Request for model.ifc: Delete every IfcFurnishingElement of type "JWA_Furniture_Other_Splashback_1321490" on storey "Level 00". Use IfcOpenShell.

First a look at what the model holds.

```python
import ifcopenshell
import ifcopenshell.util.element

model = ifcopenshell.open("model.ifc")
print(model.schema)
storey = next(s for s in model.by_type("IfcBuildingStorey") if s.Name == "Level 00")
furniture = [e for e in ifcopenshell.util.element.get_decomposition(storey) if e.is_a("IfcFurnishingElement")]
seen = {}
for e in furniture:
    element_type = ifcopenshell.util.element.get_type(e)
    name = element_type.Name if element_type not in (None, e) else None
    seen[name] = seen.get(name, 0) + 1
for name, count in sorted(seen.items(), key=str):
    print(count, "x", name)
```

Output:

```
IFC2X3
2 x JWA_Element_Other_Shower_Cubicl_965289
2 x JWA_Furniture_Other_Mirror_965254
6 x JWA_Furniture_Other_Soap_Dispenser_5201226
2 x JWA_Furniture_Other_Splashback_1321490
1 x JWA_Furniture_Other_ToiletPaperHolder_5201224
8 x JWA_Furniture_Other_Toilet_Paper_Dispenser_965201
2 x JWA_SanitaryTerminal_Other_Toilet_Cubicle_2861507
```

```python
import ifcopenshell
import ifcopenshell.api.root
import ifcopenshell.util.element

model = ifcopenshell.open("model.ifc")

storey = next(s for s in model.by_type("IfcBuildingStorey") if s.Name == "Level 00")
furniture = [e for e in ifcopenshell.util.element.get_decomposition(storey) if e.is_a("IfcFurnishingElement")]
targets = [e for e in furniture if (t := ifcopenshell.util.element.get_type(e)) not in (None, e) and t.Name == "JWA_Furniture_Other_Splashback_1321490"]

for e in targets:
    ifcopenshell.api.root.remove_product(model, product=e)
print(len(targets), "removed")

model.write("model_edited.ifc")
```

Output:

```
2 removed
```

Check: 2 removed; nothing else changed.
